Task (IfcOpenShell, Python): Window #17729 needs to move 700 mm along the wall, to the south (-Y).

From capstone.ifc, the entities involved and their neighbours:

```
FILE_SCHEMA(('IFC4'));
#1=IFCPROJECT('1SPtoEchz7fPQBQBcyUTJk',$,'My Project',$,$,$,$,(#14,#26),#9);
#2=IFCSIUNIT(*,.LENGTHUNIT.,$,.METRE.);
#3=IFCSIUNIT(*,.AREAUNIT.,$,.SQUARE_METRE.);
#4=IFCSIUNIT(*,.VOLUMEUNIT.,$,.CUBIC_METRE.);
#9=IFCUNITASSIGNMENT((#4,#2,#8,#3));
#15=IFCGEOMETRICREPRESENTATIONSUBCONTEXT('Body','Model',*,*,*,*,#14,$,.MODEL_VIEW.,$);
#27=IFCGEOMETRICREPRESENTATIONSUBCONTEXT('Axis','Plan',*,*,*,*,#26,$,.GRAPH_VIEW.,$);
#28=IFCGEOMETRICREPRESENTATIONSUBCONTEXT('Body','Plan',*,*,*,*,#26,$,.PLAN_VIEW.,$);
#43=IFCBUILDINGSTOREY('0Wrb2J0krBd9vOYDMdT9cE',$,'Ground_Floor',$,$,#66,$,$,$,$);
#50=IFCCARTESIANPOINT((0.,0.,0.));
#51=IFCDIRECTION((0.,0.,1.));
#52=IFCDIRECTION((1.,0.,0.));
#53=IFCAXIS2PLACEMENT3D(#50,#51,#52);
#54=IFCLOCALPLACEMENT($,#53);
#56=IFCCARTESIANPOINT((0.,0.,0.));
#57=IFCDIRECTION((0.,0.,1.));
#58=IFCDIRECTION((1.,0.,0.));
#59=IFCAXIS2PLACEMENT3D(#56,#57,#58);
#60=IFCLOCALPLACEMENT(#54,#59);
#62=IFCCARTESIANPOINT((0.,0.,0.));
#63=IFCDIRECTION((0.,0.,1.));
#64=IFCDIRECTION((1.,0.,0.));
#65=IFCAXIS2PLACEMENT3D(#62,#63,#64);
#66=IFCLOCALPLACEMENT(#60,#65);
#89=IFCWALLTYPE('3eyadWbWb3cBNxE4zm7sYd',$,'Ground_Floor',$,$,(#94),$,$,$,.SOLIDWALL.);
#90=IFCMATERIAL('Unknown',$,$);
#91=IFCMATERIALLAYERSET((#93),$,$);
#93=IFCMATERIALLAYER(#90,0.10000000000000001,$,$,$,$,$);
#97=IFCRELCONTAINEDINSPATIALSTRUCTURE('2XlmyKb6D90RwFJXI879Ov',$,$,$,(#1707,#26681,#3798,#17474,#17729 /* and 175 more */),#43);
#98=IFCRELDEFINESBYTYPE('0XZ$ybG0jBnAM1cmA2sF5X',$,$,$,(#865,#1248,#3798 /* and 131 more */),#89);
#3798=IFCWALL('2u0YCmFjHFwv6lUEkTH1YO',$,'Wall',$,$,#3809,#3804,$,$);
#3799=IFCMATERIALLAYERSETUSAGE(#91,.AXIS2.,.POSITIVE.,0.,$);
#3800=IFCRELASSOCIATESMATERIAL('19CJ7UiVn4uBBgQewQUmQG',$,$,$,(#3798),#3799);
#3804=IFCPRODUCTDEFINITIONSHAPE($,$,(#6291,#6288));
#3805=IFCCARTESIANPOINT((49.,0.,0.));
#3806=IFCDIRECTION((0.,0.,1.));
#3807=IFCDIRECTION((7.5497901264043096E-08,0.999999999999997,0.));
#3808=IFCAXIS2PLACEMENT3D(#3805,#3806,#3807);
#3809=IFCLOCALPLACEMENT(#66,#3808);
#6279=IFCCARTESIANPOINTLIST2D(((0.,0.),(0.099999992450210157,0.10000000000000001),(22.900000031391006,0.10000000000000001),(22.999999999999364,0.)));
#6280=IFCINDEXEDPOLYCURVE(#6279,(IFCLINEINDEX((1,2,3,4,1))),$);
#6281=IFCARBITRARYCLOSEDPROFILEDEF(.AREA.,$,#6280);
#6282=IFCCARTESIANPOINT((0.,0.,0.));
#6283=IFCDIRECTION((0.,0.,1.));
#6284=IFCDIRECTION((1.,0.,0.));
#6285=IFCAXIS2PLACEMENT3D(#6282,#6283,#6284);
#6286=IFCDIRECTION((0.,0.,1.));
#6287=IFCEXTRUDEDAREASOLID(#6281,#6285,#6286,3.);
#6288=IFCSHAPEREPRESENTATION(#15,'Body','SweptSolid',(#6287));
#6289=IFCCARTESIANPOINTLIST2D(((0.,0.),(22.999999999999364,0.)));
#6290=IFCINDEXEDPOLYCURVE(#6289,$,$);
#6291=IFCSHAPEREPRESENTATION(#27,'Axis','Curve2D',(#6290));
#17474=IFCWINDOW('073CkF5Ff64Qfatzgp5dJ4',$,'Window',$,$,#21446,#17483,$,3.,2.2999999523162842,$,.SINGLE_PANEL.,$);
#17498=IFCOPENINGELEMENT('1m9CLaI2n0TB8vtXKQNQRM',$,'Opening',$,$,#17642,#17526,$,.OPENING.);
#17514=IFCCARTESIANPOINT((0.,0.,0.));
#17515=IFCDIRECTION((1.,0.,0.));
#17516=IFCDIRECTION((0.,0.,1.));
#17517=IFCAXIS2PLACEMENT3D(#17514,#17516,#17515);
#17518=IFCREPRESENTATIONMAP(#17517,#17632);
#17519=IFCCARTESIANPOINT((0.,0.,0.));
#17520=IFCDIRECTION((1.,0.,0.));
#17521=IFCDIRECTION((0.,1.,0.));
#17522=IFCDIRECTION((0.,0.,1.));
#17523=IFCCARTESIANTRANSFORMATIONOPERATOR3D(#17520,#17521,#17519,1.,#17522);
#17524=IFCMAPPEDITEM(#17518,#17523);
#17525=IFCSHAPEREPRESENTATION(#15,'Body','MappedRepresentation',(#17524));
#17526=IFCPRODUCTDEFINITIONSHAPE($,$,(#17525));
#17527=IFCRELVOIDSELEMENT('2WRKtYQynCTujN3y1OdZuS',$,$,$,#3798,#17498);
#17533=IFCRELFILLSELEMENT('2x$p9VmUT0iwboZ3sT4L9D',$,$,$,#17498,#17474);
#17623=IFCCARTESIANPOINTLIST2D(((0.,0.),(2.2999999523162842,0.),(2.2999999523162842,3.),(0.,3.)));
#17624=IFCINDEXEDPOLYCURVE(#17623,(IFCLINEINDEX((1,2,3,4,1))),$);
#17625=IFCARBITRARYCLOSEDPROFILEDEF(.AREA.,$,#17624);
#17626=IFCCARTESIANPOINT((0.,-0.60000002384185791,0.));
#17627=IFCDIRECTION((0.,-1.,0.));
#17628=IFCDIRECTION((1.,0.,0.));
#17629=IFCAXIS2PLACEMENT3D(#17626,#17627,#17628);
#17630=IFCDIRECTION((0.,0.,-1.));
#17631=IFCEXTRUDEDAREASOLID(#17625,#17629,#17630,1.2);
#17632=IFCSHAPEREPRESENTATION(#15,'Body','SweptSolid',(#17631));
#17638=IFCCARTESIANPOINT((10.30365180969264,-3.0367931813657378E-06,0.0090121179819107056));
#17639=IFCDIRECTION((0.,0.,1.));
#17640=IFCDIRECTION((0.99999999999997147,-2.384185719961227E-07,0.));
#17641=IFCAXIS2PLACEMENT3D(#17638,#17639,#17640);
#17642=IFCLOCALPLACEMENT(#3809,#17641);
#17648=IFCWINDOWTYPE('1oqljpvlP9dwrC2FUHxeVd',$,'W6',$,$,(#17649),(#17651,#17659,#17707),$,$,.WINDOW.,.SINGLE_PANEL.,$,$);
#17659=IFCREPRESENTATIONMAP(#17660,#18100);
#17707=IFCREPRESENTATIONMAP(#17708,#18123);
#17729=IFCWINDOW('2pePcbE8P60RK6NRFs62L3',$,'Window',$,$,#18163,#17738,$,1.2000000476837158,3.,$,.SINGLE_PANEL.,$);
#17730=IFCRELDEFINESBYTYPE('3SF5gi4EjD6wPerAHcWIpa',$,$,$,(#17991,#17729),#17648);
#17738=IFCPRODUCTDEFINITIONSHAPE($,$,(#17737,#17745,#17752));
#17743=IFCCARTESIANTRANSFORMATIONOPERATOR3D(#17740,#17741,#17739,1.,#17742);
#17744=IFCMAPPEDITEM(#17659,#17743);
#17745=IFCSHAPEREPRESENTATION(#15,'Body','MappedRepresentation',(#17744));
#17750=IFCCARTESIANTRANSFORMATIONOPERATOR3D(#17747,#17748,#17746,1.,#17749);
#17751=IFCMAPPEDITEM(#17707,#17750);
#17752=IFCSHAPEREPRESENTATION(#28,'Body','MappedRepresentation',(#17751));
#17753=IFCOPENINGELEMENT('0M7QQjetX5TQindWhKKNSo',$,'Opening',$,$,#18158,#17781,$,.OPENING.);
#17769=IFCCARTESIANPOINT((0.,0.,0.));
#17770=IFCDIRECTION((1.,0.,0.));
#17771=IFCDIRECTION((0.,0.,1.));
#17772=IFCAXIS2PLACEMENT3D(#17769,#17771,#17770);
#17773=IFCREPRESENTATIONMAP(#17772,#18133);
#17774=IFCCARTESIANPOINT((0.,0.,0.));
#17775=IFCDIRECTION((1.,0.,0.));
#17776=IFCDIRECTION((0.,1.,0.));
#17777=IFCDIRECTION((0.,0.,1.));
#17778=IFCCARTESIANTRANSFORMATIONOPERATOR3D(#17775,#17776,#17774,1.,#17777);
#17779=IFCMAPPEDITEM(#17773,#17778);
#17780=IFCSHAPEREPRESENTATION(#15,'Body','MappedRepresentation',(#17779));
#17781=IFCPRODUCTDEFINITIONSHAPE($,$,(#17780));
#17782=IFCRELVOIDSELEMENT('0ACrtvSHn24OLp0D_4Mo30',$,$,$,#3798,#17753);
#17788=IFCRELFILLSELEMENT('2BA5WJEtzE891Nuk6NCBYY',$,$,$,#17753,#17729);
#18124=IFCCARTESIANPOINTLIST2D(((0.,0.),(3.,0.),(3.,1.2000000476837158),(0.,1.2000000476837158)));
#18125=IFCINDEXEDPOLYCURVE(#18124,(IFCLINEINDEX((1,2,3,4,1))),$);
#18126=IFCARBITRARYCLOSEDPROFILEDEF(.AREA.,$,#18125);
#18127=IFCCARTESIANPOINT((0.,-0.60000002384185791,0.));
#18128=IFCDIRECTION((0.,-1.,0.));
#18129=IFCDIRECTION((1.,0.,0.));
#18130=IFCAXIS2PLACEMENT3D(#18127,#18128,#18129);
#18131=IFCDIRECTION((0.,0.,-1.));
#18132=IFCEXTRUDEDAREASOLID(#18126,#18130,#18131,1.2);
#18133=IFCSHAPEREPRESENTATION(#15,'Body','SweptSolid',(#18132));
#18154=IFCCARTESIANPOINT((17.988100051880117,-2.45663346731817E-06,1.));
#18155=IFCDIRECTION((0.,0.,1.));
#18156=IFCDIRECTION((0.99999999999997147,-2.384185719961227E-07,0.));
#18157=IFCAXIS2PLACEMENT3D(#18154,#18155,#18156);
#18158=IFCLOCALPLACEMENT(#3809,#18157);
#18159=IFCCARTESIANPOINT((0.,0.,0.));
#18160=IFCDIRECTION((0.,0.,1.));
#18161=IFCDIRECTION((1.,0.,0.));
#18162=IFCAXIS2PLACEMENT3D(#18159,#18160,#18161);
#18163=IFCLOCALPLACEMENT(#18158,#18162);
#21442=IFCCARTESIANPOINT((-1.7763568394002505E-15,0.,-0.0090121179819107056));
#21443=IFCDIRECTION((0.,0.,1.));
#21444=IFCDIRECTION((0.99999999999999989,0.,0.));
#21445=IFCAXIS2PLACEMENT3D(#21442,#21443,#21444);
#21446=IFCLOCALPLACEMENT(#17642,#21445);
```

```python
import ifcopenshell
import ifcopenshell.api.geometry
import ifcopenshell.util.placement
import ifcopenshell.util.unit

model = ifcopenshell.open("capstone.ifc")
unit_scale = ifcopenshell.util.unit.calculate_unit_scale(model)

window = model.by_id(17729)
opening = window.FillsVoids[0].RelatingOpeningElement
wall = opening.VoidsElements[0].RelatingBuildingElement

wall_matrix = ifcopenshell.util.placement.get_local_placement(wall.ObjectPlacement)
shift = wall_matrix[:3, 0] * -0.7 / unit_scale
before = ifcopenshell.util.placement.get_local_placement(window.ObjectPlacement)[:3, 3].copy()

# The window is placed relative to its opening, so it follows when the opening moves.
matrix = ifcopenshell.util.placement.get_local_placement(opening.ObjectPlacement)
matrix[:3, 3] += shift
ifcopenshell.api.geometry.edit_object_placement(
    model, product=opening, matrix=matrix, is_si=False, should_transform_children=True
)

after = ifcopenshell.util.placement.get_local_placement(window.ObjectPlacement)[:3, 3]
print("window moved by", (after - before).round(3) + 0.0)

model.write("capstone-out.ifc")
```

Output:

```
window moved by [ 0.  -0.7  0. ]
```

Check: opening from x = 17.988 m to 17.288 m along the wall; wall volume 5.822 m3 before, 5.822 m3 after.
